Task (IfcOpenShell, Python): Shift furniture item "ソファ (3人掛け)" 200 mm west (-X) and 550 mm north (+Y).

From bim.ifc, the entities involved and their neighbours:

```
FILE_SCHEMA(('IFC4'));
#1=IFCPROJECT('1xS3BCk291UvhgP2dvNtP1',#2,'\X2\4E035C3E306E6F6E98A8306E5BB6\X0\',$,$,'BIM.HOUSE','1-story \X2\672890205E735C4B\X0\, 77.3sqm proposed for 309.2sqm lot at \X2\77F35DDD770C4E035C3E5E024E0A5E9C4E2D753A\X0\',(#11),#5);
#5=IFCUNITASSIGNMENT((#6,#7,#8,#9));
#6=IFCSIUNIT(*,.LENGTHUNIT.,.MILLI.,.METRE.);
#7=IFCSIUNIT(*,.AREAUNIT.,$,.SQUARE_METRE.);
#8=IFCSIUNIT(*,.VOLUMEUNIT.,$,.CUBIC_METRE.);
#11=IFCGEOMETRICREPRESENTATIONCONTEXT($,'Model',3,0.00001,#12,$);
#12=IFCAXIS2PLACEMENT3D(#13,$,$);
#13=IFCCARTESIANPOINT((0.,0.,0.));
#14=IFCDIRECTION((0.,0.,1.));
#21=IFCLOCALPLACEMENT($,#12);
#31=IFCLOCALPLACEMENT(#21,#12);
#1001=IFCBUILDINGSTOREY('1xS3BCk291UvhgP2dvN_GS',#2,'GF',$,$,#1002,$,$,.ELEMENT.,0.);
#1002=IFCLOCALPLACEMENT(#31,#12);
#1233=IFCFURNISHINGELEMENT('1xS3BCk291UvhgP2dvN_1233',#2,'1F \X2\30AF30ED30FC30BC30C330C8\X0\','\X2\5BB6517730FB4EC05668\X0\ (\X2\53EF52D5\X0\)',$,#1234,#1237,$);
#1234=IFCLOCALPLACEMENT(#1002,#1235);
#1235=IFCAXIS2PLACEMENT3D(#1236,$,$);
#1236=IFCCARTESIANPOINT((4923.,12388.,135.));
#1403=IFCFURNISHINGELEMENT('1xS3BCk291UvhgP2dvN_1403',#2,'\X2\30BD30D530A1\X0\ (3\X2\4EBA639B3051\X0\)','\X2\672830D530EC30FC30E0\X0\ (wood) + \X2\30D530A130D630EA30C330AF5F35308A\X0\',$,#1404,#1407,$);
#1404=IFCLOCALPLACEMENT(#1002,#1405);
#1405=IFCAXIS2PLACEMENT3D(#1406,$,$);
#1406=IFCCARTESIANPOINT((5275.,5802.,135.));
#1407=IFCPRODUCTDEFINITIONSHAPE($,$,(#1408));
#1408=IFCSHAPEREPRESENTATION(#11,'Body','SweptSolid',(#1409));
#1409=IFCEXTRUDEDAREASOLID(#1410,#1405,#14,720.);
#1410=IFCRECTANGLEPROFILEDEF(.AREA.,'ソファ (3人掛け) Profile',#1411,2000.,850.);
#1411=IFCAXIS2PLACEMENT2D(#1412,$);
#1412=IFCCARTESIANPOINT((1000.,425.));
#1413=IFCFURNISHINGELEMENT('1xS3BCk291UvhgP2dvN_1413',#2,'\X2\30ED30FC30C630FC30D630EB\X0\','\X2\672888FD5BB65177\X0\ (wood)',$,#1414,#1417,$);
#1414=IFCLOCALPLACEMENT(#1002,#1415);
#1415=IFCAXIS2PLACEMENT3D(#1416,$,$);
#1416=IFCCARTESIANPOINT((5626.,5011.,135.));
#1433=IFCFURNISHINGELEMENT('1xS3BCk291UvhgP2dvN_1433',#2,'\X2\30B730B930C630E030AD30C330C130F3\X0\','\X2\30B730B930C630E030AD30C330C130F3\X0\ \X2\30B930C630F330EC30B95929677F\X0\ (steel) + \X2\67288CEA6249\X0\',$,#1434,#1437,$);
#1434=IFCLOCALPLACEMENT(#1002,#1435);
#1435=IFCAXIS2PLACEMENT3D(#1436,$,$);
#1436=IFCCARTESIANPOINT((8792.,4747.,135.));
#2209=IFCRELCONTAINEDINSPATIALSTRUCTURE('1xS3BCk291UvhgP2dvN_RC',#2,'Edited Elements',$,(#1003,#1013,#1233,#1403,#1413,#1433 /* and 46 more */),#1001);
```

```python
import ifcopenshell
import ifcopenshell.api.geometry
import ifcopenshell.util.placement
import ifcopenshell.util.unit

model = ifcopenshell.open("bim.ifc")
unit_scale = ifcopenshell.util.unit.calculate_unit_scale(model)

item = model.by_guid("1xS3BCk291UvhgP2dvN_1403")
matrix = ifcopenshell.util.placement.get_local_placement(item.ObjectPlacement)
matrix[0, 3] -= 0.2 / unit_scale
matrix[1, 3] += 0.55 / unit_scale
ifcopenshell.api.geometry.edit_object_placement(model, product=item, matrix=matrix, is_si=False)

print(ifcopenshell.util.placement.get_local_placement(item.ObjectPlacement).round(3) + 0.0)

model.write("bim-out.ifc")
```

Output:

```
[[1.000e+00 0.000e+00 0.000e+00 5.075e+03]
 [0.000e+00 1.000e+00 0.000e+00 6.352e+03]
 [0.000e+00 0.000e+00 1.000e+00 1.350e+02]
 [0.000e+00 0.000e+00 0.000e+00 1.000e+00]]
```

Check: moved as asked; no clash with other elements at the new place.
